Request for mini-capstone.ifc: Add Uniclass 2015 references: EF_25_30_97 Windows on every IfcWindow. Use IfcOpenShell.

First a look at what the model holds.

```python
import ifcopenshell

model = ifcopenshell.open("mini-capstone.ifc")
print(model.schema)
print("classifications:", [c.Name for c in model.by_type("IfcClassification")])
for ifc_class in ("IfcDoor", "IfcRoof", "IfcStair", "IfcWall", "IfcWindow"):
    print(ifc_class, len(model.by_type(ifc_class)))
```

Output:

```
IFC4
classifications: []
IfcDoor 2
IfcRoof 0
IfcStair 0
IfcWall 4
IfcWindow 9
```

```python
import ifcopenshell
import ifcopenshell.api.classification

model = ifcopenshell.open("mini-capstone.ifc")

system = ifcopenshell.api.classification.add_classification(model, classification="Uniclass 2015")

codes = {
    "IfcWindow": ("EF_25_30_97", "Windows"),
}
for ifc_class, (code, name) in codes.items():
    products = model.by_type(ifc_class)
    ifcopenshell.api.classification.add_reference(
        model, products=products, classification=system, identification=code, name=name
    )
    print(code, len(products))

model.write("mini-capstone_edited.ifc")
```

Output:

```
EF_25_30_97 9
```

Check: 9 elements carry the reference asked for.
